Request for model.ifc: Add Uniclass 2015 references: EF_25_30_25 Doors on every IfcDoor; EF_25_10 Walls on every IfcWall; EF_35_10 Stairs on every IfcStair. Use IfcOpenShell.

First a look at what the model holds.

```python
import ifcopenshell

model = ifcopenshell.open("model.ifc")
print(model.schema)
print("classifications:", [c.Name for c in model.by_type("IfcClassification")])
for ifc_class in ("IfcDoor", "IfcRoof", "IfcStair", "IfcWall", "IfcWindow"):
    print(ifc_class, len(model.by_type(ifc_class)))
```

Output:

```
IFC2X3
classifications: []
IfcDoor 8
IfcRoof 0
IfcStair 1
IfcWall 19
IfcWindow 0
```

```python
import ifcopenshell
import ifcopenshell.api.classification

model = ifcopenshell.open("model.ifc")

# IFC2X3 requires Source and Edition and has no link from the project to the system.
system = model.create_entity("IfcClassification", Source="NBS", Edition="2015", Name="Uniclass 2015")

codes = {
    "IfcDoor": ("EF_25_30_25", "Doors"),
    "IfcWall": ("EF_25_10", "Walls"),
    "IfcStair": ("EF_35_10", "Stairs"),
}
for ifc_class, (code, name) in codes.items():
    products = model.by_type(ifc_class)
    ifcopenshell.api.classification.add_reference(
        model, products=products, classification=system, identification=code, name=name
    )
    print(code, len(products))

model.write("model-out.ifc")
```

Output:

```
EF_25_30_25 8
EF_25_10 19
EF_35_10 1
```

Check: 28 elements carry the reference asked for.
